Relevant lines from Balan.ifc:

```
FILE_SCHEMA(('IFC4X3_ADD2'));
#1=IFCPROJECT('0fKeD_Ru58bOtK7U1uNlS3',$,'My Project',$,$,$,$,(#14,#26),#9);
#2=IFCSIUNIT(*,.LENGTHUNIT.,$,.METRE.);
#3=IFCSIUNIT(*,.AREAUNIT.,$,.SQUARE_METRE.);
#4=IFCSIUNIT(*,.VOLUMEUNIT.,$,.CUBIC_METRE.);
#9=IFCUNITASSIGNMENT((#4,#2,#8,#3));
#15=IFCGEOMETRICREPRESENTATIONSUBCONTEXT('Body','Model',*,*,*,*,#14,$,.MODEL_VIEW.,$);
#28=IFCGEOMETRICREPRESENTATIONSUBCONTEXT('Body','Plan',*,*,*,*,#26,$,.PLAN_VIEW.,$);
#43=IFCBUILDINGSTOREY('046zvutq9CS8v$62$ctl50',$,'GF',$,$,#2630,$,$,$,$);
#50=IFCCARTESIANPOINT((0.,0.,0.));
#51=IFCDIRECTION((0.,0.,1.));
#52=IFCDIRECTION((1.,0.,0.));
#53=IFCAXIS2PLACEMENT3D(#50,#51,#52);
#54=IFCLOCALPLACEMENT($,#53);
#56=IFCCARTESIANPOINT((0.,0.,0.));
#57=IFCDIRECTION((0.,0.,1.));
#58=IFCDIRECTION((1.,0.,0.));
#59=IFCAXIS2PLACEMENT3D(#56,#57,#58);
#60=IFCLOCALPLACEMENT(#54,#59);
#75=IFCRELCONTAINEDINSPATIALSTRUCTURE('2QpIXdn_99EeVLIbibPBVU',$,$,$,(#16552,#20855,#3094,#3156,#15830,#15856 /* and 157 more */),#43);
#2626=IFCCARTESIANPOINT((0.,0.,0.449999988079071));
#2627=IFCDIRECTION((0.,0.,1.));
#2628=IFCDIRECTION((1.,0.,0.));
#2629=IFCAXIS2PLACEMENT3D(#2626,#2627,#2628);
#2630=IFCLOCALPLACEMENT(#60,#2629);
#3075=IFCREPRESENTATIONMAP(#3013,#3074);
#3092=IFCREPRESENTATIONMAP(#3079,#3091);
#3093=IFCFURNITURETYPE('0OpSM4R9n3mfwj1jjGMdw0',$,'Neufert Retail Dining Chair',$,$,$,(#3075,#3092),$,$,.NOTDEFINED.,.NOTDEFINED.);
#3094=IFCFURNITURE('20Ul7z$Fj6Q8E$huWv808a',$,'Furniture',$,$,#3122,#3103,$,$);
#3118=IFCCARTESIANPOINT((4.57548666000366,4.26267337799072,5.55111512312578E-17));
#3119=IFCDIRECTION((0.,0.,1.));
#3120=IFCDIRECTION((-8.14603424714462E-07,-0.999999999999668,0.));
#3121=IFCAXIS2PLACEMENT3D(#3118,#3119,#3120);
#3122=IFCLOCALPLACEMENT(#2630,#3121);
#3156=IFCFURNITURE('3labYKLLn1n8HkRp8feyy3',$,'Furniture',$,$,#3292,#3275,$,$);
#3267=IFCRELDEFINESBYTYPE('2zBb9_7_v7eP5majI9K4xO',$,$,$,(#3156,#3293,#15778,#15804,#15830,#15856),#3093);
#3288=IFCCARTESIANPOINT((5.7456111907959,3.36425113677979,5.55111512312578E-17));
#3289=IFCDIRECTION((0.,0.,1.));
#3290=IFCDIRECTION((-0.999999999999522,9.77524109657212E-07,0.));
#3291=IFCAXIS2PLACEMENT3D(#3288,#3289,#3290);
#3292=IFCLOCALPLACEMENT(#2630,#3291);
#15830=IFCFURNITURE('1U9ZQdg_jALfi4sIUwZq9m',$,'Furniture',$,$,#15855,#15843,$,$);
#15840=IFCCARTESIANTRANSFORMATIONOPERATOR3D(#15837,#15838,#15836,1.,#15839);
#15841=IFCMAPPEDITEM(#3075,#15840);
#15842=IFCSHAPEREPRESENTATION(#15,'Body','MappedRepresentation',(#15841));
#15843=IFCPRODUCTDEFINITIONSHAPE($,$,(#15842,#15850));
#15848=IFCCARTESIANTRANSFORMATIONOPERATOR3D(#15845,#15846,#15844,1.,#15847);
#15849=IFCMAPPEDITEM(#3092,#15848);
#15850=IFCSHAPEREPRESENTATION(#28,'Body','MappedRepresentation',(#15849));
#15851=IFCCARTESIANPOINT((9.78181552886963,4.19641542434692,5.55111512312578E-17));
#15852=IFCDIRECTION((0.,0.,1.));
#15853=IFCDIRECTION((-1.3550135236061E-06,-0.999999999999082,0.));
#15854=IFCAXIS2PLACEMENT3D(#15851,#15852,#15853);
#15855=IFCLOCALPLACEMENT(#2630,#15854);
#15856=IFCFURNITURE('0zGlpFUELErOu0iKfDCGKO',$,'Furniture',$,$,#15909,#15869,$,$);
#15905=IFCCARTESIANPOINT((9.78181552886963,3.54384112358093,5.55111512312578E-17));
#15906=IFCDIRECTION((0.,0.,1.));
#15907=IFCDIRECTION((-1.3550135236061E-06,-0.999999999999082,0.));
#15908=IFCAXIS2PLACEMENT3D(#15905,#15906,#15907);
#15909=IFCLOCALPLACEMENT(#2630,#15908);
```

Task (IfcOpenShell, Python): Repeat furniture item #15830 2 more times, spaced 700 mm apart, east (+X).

```python
import numpy as np
import ifcopenshell
import ifcopenshell.api.geometry
import ifcopenshell.api.root
import ifcopenshell.util.element
import ifcopenshell.util.placement

model = ifcopenshell.open("Balan.ifc")

source = model.by_id(15830)
base = ifcopenshell.util.placement.get_local_placement(source.ObjectPlacement)
step = np.array([1.0, 0.0, 0.0]) * 0.7

for i in range(1, 3):
    copy = ifcopenshell.api.root.copy_class(model, product=source)
    copy.Representation = ifcopenshell.util.element.copy_deep(
        model, source.Representation, exclude=["IfcGeometricRepresentationContext", "IfcRepresentationMap"]
    )
    matrix = base.copy()
    matrix[:3, 3] += i * step
    print("added at", matrix[:3, 3].round(3) + 0.0)
    ifcopenshell.api.geometry.edit_object_placement(model, product=copy, matrix=matrix, is_si=False)

model.write("Balan_updated.ifc")
```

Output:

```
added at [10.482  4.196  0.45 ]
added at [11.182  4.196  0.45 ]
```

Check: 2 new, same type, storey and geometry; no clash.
